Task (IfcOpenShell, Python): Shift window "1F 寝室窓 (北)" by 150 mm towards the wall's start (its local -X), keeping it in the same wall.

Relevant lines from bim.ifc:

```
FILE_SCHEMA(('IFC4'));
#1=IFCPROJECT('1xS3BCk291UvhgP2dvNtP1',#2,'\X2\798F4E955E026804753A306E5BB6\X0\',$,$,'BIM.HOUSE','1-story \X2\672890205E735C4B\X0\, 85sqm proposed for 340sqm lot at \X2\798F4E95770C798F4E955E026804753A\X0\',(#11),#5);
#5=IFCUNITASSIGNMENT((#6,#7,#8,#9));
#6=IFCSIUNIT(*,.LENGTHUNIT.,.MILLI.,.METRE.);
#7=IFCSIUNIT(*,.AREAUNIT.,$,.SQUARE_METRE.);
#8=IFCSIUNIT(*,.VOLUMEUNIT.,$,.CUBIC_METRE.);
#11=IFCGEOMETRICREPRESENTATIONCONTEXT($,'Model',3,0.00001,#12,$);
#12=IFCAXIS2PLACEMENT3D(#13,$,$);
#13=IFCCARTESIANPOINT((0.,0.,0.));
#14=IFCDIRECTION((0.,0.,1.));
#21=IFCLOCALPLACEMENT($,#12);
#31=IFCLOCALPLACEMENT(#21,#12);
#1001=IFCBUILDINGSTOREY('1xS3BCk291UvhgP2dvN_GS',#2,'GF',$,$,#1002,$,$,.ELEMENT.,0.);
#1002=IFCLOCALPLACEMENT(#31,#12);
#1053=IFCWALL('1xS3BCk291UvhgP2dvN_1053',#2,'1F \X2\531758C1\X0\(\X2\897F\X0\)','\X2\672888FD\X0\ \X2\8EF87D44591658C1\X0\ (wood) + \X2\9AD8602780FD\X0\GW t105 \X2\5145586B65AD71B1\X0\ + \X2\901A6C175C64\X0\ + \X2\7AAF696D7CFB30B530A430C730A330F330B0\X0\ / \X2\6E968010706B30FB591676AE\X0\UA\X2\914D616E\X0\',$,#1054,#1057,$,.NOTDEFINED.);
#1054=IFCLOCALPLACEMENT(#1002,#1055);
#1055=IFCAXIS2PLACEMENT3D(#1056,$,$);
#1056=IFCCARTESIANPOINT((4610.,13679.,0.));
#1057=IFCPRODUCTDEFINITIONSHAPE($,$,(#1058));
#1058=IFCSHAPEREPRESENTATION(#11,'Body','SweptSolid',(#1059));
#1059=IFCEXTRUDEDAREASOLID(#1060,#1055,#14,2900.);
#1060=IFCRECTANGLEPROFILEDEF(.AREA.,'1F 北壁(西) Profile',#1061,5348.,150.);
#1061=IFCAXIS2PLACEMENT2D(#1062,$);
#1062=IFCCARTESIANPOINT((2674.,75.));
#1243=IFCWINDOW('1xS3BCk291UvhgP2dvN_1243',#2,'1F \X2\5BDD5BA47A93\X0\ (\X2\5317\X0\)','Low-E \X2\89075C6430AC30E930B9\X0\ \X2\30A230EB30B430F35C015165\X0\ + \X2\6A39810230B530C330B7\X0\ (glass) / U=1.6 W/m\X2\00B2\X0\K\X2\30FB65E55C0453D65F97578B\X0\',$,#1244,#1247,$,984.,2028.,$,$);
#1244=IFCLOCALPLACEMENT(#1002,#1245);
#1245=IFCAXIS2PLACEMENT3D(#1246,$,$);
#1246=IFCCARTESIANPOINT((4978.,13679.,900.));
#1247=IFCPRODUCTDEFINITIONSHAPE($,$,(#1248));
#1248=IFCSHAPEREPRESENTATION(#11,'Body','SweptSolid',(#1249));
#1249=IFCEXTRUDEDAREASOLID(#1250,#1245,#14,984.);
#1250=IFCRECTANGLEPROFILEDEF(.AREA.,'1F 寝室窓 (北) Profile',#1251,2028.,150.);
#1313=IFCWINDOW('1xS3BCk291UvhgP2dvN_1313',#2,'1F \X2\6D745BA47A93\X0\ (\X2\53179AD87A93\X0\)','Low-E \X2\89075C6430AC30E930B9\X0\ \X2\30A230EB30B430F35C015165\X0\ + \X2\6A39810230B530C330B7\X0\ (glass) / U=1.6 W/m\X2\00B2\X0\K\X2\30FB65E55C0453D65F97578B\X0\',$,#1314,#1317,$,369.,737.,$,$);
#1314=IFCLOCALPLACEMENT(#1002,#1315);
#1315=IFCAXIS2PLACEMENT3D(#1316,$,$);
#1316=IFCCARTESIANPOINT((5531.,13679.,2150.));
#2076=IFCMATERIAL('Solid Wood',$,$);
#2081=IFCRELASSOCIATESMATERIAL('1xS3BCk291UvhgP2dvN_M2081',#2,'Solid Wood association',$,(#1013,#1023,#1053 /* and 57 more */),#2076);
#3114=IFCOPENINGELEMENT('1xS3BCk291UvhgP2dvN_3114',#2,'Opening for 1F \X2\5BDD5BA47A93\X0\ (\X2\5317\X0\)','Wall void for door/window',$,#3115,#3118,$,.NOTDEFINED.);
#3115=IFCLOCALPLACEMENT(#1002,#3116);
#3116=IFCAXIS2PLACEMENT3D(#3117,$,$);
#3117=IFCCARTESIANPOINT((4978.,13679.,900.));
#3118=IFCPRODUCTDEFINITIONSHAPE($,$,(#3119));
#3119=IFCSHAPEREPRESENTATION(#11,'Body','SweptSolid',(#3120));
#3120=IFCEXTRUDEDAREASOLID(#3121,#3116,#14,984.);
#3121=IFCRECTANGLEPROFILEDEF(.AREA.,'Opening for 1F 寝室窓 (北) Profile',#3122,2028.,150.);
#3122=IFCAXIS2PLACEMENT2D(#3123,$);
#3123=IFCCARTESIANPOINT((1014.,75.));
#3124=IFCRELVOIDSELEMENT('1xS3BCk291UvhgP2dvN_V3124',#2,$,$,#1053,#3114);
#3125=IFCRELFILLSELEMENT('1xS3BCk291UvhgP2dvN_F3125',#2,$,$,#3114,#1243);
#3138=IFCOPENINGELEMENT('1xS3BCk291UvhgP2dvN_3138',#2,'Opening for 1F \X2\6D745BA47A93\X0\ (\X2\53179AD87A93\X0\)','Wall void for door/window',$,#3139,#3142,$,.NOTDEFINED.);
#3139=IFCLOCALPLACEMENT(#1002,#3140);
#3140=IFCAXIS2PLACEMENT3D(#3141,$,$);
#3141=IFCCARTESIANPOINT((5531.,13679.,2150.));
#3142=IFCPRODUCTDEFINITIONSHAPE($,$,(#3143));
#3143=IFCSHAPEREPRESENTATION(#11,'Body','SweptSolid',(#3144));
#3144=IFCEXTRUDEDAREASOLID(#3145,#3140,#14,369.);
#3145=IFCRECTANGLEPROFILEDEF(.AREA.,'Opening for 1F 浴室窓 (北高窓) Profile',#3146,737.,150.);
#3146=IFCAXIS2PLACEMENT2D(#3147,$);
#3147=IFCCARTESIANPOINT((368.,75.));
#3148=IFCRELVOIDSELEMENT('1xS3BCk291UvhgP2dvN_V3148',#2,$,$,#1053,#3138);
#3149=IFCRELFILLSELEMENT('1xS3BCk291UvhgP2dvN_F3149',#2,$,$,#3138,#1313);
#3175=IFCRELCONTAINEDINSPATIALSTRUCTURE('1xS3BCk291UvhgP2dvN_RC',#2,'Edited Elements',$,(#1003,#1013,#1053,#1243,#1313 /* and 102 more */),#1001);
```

```python
import ifcopenshell
import ifcopenshell.api.geometry
import ifcopenshell.util.placement

model = ifcopenshell.open("bim.ifc")

window = model.by_guid("1xS3BCk291UvhgP2dvN_1243")
opening = window.FillsVoids[0].RelatingOpeningElement
wall = opening.VoidsElements[0].RelatingBuildingElement

wall_matrix = ifcopenshell.util.placement.get_local_placement(wall.ObjectPlacement)
shift = wall_matrix[:3, 0] * -150.0
before = ifcopenshell.util.placement.get_local_placement(window.ObjectPlacement)[:3, 3].copy()

# The window is not placed relative to its opening, so move both.
for product in (opening, window):
    matrix = ifcopenshell.util.placement.get_local_placement(product.ObjectPlacement)
    matrix[:3, 3] += shift
    ifcopenshell.api.geometry.edit_object_placement(model, product=product, matrix=matrix, is_si=False)

after = ifcopenshell.util.placement.get_local_placement(window.ObjectPlacement)[:3, 3]
print("window moved by", (after - before).round(3) + 0.0)

model.write("bim_edited.ifc")
```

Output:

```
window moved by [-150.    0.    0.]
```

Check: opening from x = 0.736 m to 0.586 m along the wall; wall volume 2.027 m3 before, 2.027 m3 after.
